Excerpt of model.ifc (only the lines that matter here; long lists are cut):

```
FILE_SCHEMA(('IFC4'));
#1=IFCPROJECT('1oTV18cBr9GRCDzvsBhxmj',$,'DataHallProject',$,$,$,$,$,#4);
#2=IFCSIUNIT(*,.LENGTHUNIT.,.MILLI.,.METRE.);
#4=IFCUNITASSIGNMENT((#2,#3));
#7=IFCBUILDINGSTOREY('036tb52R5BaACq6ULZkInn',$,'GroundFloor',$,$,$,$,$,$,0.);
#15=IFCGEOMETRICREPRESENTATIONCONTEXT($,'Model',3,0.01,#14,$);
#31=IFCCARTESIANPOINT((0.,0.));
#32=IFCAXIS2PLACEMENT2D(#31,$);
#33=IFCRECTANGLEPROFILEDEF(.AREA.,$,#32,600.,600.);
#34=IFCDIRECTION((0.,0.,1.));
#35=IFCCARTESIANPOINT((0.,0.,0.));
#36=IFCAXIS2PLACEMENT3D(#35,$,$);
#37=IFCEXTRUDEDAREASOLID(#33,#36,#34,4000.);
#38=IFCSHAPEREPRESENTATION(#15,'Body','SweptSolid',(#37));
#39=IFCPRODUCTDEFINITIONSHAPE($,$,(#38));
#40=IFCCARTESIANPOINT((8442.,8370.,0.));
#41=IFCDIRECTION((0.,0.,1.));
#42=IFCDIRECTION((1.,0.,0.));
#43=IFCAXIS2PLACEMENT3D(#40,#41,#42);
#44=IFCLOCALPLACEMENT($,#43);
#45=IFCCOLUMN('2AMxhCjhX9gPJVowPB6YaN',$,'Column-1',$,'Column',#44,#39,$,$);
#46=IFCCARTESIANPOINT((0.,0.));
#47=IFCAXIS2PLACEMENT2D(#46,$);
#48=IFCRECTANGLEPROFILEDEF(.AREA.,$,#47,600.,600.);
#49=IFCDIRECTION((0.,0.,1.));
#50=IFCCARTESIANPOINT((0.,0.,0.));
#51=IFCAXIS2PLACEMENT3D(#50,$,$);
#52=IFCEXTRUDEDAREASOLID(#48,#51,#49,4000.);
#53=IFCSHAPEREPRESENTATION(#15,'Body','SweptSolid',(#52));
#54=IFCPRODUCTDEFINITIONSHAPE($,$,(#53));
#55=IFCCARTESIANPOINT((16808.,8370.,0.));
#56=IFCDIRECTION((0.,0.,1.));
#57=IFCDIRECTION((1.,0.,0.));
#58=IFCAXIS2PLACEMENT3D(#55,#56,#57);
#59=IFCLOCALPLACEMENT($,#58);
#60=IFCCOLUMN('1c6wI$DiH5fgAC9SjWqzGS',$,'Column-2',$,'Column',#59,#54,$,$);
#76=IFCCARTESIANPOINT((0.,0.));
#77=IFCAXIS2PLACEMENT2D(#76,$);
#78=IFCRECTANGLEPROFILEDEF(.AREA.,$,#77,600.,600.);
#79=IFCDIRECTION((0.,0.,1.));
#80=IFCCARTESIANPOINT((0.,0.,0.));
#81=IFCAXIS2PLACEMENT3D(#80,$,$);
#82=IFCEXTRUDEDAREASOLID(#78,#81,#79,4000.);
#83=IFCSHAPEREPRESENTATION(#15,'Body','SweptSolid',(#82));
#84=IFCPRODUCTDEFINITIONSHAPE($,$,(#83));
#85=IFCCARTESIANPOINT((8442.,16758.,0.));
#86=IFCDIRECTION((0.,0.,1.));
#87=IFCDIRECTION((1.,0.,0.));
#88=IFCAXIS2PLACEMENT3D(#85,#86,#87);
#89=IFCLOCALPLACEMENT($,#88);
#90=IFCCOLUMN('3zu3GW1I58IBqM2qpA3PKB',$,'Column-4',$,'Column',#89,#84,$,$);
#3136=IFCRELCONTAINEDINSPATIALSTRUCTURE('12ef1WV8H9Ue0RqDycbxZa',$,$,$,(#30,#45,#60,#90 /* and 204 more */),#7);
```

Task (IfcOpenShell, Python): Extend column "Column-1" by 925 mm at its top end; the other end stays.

```python
import ifcopenshell
import ifcopenshell.util.unit

model = ifcopenshell.open("model.ifc")
unit_scale = ifcopenshell.util.unit.calculate_unit_scale(model)

member = model.by_id(45)
change = 0.925 / unit_scale

# The extrusion runs towards the end named, so only its depth changes.
body = next(r for r in member.Representation.Representations if r.RepresentationIdentifier == "Body")
solid = body.Items[0]
old_length = solid.Depth
solid.Depth += change

print(f"length {old_length:g} -> {solid.Depth:g}")

model.write("model_edited.ifc")
```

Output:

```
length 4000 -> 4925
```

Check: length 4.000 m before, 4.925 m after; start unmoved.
